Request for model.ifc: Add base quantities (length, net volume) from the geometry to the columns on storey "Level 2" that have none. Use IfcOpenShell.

First a look at what the model holds.

```python
import ifcopenshell
import ifcopenshell.util.element
import ifcopenshell.util.unit

model = ifcopenshell.open("model.ifc")
print(model.schema)
for unit_type in ("LENGTHUNIT", "AREAUNIT", "VOLUMEUNIT"):
    print(unit_type, ifcopenshell.util.unit.calculate_unit_scale(model, unit_type))
storey = next(s for s in model.by_type("IfcBuildingStorey") if s.Name == "Level 2")
columns = [e for e in ifcopenshell.util.element.get_decomposition(storey) if e.is_a("IfcColumn")]
for e in sorted(columns, key=lambda e: e.id()):
    print(e.id(), e.is_a(), e.Name, list(ifcopenshell.util.element.get_psets(e, qtos_only=True)), sep=" | ")
```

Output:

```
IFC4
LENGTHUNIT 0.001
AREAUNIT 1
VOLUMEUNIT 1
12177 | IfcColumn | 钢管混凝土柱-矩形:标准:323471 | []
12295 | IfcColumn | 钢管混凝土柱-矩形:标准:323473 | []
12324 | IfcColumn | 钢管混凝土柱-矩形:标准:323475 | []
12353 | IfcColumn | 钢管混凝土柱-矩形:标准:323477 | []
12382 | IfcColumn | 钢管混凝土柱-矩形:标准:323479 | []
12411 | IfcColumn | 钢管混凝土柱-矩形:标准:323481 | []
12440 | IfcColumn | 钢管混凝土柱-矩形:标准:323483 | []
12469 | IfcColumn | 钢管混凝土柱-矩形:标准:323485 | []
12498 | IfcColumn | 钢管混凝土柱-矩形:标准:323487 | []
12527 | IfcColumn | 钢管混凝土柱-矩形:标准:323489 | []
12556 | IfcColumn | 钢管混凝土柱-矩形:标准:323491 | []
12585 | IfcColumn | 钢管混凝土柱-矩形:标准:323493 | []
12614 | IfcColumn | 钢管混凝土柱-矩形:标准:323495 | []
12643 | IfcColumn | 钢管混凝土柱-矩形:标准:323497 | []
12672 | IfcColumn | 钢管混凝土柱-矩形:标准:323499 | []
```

```python
import ifcopenshell
import ifcopenshell.api.pset
import ifcopenshell.geom
import ifcopenshell.util.element
import ifcopenshell.util.shape
import ifcopenshell.util.unit

model = ifcopenshell.open("model.ifc")
unit_scale = ifcopenshell.util.unit.calculate_unit_scale(model)
volume_scale = ifcopenshell.util.unit.calculate_unit_scale(model, "VOLUMEUNIT")
settings = ifcopenshell.geom.settings()

storey = next(s for s in model.by_type("IfcBuildingStorey") if s.Name == "Level 2")
columns = [e for e in ifcopenshell.util.element.get_decomposition(storey) if e.is_a("IfcColumn")]

for e in sorted(columns, key=lambda e: e.id()):
    if ifcopenshell.util.element.get_psets(e, qtos_only=True, should_inherit=False):
        continue
    # Geometry comes back in metres, in the element's own axes.
    shape = ifcopenshell.geom.create_shape(settings, e)
    values = {
        "Length": ifcopenshell.util.shape.get_z(shape.geometry) / unit_scale,
        "NetVolume": ifcopenshell.util.shape.get_volume(shape.geometry) / volume_scale,
    }
    qto = ifcopenshell.api.pset.add_qto(model, product=e, name="Qto_ColumnBaseQuantities")
    ifcopenshell.api.pset.edit_qto(model, qto=qto, properties=values)
    print(e.id(), {k: round(v, 3) for k, v in values.items()})

model.write("model_rev.ifc")
```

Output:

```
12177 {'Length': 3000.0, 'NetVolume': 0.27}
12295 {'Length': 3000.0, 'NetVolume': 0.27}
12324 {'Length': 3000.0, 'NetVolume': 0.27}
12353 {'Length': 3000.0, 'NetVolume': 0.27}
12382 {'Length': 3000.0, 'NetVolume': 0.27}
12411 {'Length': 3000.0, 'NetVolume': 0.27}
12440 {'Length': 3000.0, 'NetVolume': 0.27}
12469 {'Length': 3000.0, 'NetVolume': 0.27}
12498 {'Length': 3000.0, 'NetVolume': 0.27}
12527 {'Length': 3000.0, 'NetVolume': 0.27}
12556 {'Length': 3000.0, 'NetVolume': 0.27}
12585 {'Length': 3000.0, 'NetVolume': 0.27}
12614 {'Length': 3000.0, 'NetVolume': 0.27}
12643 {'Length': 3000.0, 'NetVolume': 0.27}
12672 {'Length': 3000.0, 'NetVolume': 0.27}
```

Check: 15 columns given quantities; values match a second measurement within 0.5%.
